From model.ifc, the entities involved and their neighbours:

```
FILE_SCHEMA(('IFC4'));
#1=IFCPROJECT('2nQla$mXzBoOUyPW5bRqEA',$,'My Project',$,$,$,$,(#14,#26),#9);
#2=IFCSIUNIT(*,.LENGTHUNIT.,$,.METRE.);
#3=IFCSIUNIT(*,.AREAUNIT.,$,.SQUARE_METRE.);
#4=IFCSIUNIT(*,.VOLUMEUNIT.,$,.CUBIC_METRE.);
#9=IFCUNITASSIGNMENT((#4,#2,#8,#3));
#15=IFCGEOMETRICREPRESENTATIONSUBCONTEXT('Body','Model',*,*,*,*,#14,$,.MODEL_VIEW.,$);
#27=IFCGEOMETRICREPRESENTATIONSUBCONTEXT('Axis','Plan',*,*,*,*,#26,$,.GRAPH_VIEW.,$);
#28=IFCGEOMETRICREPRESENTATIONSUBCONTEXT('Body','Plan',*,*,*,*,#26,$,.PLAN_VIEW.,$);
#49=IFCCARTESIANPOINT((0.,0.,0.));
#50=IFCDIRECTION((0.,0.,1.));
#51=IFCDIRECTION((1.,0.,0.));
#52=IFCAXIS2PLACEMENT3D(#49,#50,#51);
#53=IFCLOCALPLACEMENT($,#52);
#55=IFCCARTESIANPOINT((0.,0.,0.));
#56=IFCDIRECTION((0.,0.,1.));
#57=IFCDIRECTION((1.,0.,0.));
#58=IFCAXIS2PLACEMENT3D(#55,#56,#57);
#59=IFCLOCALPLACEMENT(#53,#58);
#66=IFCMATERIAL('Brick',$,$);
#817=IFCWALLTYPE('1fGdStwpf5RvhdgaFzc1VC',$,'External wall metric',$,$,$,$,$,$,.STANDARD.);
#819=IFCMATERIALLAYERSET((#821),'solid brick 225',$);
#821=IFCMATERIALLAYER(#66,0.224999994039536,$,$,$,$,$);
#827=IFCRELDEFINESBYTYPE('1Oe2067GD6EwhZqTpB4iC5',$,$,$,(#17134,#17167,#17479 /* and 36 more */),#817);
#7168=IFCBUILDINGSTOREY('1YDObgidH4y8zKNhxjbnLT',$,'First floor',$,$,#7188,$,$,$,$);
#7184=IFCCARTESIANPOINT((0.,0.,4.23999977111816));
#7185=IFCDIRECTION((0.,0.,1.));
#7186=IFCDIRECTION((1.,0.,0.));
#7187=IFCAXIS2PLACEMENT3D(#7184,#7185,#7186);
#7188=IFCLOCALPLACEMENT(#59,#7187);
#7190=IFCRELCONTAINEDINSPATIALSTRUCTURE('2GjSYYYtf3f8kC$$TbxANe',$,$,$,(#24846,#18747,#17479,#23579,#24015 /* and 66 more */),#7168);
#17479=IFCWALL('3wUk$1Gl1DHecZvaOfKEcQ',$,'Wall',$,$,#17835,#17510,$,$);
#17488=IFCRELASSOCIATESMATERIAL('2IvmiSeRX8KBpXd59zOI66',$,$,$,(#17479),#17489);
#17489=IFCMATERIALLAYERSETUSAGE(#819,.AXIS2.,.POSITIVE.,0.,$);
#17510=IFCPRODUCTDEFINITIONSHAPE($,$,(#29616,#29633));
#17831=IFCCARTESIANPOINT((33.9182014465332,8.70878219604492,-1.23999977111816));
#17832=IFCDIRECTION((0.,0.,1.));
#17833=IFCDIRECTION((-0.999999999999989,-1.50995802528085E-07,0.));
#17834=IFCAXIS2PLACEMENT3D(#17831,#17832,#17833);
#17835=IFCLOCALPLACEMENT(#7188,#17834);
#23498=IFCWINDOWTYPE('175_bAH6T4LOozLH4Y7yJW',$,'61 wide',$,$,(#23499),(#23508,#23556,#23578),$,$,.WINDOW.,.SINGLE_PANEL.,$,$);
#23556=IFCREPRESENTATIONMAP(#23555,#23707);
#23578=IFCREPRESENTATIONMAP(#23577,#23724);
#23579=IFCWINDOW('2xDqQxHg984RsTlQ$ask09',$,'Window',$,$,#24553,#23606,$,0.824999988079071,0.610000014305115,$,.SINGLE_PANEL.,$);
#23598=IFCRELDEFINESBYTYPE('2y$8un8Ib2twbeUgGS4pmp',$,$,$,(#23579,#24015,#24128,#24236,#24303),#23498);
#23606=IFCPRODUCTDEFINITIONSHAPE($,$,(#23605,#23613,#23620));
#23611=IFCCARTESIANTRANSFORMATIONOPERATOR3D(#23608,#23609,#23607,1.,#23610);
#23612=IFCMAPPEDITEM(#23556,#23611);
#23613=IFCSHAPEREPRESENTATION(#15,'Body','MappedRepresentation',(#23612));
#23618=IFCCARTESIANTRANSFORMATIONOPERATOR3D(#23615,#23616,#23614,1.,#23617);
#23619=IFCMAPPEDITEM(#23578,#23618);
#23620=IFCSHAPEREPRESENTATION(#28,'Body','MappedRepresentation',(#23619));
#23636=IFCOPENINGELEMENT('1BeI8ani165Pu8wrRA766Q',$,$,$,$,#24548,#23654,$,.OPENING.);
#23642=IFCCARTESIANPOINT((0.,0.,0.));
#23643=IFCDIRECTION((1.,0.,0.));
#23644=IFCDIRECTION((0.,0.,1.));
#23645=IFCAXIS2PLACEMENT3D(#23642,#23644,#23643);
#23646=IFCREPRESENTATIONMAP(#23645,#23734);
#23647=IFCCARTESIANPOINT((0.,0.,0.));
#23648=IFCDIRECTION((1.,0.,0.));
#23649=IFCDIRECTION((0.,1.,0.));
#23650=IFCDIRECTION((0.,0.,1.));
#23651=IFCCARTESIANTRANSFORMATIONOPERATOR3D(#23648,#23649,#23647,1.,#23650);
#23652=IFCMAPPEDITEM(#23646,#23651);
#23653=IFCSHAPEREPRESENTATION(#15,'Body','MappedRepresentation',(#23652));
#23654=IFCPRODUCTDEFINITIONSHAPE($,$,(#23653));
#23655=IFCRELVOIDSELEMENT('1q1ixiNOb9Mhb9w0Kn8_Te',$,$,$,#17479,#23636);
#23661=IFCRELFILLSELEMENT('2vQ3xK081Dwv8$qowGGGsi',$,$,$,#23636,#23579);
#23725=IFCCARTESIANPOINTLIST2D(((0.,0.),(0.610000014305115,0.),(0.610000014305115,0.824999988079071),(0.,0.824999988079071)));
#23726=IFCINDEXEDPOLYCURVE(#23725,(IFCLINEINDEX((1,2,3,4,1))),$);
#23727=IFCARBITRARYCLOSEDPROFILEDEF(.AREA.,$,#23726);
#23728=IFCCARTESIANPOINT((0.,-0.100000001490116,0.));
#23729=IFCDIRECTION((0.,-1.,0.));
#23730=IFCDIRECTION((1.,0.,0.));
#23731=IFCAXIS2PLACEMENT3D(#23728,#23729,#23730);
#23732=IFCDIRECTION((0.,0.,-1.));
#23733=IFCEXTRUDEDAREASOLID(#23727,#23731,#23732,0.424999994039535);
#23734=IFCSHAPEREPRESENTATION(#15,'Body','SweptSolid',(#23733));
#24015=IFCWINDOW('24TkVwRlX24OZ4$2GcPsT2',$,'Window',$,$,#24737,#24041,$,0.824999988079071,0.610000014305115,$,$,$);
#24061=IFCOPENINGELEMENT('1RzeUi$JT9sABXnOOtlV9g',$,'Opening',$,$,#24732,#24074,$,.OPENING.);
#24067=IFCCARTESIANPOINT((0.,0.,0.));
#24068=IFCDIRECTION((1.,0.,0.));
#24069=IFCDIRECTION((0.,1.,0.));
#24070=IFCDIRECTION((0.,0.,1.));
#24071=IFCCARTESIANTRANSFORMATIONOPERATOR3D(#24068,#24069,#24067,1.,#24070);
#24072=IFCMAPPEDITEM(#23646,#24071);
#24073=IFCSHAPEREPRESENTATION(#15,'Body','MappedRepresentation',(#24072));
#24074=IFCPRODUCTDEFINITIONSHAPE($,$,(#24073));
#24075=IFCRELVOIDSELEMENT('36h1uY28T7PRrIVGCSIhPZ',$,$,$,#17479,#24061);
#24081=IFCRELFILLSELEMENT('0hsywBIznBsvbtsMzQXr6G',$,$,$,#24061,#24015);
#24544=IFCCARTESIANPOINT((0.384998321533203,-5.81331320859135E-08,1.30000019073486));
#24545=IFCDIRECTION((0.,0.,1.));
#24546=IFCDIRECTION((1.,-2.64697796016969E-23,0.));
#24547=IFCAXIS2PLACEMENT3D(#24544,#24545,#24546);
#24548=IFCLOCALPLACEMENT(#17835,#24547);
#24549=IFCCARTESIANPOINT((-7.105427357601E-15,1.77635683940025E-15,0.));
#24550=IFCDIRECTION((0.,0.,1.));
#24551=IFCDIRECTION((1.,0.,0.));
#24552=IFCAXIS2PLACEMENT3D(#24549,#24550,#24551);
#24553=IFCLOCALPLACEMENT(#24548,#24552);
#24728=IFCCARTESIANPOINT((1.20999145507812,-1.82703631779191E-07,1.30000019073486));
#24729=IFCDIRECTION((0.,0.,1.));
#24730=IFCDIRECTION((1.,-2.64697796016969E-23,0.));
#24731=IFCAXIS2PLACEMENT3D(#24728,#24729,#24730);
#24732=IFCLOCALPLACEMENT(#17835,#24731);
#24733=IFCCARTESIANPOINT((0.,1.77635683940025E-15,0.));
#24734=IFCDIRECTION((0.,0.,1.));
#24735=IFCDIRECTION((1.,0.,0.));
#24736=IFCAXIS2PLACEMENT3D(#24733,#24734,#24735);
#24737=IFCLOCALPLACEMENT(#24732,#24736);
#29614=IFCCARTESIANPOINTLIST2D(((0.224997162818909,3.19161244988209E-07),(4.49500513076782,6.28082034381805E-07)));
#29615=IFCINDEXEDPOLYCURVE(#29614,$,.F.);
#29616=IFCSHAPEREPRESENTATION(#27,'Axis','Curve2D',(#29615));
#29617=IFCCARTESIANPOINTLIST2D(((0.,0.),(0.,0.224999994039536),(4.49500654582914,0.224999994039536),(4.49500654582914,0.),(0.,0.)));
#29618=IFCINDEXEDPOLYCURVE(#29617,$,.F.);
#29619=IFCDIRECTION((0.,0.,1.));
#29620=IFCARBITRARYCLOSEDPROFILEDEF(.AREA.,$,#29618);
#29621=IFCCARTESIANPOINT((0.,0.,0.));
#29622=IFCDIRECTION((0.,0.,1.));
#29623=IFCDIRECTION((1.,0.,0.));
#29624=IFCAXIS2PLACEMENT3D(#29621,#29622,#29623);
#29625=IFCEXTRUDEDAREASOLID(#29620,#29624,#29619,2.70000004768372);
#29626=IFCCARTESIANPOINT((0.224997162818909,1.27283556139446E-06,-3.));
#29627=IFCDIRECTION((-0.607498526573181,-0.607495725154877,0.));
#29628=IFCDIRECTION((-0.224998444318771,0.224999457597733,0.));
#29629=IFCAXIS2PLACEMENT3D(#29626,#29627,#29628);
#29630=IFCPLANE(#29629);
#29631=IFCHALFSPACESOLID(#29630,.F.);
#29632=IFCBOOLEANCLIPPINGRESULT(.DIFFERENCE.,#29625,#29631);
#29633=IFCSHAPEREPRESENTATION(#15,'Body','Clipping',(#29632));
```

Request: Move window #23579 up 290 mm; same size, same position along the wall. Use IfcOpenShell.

```python
import numpy as np
import ifcopenshell
import ifcopenshell.api.geometry
import ifcopenshell.util.placement
import ifcopenshell.util.unit

model = ifcopenshell.open("model.ifc")
unit_scale = ifcopenshell.util.unit.calculate_unit_scale(model)

window = model.by_guid("2xDqQxHg984RsTlQ$ask09")
opening = window.FillsVoids[0].RelatingOpeningElement
dz = 0.29 / unit_scale

shift = np.array([0.0, 0.0, dz])
# The window is placed relative to its opening, so it follows when the opening moves.
matrix = ifcopenshell.util.placement.get_local_placement(opening.ObjectPlacement)
matrix[:3, 3] += shift
ifcopenshell.api.geometry.edit_object_placement(
    model, product=opening, matrix=matrix, is_si=False, should_transform_children=True
)

print(f"moved by {dz * unit_scale:+.3f} m")

model.write("model_rev.ifc")
```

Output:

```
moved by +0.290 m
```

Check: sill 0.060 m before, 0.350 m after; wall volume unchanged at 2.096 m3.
